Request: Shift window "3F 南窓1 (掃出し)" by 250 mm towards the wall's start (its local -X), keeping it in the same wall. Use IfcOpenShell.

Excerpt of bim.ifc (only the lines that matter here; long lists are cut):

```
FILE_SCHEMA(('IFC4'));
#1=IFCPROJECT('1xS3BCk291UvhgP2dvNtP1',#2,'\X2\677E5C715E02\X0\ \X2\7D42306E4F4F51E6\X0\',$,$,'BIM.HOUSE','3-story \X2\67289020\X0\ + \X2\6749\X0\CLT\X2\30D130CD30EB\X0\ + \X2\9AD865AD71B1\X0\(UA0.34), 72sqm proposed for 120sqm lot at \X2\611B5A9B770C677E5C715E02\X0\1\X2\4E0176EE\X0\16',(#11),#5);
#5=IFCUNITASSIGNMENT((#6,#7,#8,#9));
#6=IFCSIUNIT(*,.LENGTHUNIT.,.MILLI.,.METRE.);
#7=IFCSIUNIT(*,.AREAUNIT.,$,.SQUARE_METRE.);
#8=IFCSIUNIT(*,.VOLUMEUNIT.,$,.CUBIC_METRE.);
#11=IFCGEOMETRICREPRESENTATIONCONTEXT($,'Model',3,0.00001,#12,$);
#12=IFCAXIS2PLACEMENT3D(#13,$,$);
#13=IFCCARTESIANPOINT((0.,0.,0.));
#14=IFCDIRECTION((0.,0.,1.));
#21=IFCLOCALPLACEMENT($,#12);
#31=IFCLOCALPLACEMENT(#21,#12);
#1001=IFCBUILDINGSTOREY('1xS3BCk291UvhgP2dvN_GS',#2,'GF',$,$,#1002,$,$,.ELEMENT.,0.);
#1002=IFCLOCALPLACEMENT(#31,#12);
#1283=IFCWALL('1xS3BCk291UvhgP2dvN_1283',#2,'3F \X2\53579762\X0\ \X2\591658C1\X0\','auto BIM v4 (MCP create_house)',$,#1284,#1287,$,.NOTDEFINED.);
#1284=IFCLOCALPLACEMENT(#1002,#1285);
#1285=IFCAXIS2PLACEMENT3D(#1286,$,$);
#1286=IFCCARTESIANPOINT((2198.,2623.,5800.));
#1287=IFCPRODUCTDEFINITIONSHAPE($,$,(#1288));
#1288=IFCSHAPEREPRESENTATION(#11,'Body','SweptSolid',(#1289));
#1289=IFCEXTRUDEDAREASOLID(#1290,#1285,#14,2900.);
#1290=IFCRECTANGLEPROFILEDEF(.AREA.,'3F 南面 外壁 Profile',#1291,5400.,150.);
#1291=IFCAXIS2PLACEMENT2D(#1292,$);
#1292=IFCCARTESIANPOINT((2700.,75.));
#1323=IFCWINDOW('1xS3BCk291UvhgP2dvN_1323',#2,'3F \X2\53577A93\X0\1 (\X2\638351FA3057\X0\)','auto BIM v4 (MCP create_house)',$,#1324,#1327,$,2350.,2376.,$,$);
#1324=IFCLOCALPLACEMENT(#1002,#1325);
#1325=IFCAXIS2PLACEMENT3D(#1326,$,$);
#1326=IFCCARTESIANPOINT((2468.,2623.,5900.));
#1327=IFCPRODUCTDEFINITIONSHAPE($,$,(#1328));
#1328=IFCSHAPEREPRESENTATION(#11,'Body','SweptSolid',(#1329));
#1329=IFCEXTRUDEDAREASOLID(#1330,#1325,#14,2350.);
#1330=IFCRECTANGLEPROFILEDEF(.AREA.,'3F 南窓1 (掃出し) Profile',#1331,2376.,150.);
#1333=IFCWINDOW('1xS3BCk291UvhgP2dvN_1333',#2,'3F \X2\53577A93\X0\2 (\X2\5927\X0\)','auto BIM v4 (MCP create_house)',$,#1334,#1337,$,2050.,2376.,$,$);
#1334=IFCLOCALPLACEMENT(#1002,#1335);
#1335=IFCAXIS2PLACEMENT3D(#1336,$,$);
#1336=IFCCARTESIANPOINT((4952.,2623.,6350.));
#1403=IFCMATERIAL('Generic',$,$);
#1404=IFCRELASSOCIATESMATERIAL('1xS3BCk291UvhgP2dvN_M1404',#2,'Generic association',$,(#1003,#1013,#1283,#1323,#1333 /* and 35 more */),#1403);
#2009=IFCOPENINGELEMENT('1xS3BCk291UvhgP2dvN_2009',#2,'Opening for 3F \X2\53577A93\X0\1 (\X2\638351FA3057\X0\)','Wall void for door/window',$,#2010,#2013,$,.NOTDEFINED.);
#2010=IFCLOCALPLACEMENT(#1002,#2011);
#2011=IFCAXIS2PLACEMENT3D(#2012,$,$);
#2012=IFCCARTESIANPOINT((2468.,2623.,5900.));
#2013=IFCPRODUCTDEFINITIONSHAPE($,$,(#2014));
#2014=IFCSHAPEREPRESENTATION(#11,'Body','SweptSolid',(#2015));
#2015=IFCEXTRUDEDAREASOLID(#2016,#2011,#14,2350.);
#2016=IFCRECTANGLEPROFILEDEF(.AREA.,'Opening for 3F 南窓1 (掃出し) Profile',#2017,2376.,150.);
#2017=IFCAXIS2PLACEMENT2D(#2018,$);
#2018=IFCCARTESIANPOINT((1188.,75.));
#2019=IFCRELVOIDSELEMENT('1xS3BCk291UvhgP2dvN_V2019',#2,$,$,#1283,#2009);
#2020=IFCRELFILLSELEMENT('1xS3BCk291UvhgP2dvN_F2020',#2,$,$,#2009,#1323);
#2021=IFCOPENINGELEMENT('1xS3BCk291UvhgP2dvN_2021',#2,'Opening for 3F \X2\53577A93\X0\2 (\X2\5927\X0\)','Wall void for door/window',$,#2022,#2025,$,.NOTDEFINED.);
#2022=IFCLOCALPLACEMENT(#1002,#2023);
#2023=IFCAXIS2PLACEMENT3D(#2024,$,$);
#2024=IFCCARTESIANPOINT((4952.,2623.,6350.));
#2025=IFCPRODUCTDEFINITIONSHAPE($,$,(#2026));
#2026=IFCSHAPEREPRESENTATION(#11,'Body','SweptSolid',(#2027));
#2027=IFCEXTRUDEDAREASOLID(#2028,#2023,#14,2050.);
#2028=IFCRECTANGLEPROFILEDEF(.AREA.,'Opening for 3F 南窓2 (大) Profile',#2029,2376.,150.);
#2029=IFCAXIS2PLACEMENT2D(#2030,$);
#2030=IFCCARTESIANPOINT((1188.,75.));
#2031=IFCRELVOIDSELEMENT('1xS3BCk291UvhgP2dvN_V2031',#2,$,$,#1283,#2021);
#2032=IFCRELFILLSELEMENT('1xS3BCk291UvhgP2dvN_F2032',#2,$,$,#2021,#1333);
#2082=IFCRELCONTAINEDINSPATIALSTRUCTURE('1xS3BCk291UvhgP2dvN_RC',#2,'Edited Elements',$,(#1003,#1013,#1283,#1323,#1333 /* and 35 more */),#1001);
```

```python
import ifcopenshell
import ifcopenshell.api.geometry
import ifcopenshell.util.placement
import ifcopenshell.util.unit

model = ifcopenshell.open("bim.ifc")
unit_scale = ifcopenshell.util.unit.calculate_unit_scale(model)

window = model.by_guid("1xS3BCk291UvhgP2dvN_1323")
opening = window.FillsVoids[0].RelatingOpeningElement
wall = opening.VoidsElements[0].RelatingBuildingElement

wall_matrix = ifcopenshell.util.placement.get_local_placement(wall.ObjectPlacement)
shift = wall_matrix[:3, 0] * -0.25 / unit_scale
before = ifcopenshell.util.placement.get_local_placement(window.ObjectPlacement)[:3, 3].copy()

# The window is not placed relative to its opening, so move both.
for product in (opening, window):
    matrix = ifcopenshell.util.placement.get_local_placement(product.ObjectPlacement)
    matrix[:3, 3] += shift
    ifcopenshell.api.geometry.edit_object_placement(model, product=product, matrix=matrix, is_si=False)

after = ifcopenshell.util.placement.get_local_placement(window.ObjectPlacement)[:3, 3]
print("window moved by", (after - before).round(3) + 0.0)

model.write("bim_rev.ifc")
```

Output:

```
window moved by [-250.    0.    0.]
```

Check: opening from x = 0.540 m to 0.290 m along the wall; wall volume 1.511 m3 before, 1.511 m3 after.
